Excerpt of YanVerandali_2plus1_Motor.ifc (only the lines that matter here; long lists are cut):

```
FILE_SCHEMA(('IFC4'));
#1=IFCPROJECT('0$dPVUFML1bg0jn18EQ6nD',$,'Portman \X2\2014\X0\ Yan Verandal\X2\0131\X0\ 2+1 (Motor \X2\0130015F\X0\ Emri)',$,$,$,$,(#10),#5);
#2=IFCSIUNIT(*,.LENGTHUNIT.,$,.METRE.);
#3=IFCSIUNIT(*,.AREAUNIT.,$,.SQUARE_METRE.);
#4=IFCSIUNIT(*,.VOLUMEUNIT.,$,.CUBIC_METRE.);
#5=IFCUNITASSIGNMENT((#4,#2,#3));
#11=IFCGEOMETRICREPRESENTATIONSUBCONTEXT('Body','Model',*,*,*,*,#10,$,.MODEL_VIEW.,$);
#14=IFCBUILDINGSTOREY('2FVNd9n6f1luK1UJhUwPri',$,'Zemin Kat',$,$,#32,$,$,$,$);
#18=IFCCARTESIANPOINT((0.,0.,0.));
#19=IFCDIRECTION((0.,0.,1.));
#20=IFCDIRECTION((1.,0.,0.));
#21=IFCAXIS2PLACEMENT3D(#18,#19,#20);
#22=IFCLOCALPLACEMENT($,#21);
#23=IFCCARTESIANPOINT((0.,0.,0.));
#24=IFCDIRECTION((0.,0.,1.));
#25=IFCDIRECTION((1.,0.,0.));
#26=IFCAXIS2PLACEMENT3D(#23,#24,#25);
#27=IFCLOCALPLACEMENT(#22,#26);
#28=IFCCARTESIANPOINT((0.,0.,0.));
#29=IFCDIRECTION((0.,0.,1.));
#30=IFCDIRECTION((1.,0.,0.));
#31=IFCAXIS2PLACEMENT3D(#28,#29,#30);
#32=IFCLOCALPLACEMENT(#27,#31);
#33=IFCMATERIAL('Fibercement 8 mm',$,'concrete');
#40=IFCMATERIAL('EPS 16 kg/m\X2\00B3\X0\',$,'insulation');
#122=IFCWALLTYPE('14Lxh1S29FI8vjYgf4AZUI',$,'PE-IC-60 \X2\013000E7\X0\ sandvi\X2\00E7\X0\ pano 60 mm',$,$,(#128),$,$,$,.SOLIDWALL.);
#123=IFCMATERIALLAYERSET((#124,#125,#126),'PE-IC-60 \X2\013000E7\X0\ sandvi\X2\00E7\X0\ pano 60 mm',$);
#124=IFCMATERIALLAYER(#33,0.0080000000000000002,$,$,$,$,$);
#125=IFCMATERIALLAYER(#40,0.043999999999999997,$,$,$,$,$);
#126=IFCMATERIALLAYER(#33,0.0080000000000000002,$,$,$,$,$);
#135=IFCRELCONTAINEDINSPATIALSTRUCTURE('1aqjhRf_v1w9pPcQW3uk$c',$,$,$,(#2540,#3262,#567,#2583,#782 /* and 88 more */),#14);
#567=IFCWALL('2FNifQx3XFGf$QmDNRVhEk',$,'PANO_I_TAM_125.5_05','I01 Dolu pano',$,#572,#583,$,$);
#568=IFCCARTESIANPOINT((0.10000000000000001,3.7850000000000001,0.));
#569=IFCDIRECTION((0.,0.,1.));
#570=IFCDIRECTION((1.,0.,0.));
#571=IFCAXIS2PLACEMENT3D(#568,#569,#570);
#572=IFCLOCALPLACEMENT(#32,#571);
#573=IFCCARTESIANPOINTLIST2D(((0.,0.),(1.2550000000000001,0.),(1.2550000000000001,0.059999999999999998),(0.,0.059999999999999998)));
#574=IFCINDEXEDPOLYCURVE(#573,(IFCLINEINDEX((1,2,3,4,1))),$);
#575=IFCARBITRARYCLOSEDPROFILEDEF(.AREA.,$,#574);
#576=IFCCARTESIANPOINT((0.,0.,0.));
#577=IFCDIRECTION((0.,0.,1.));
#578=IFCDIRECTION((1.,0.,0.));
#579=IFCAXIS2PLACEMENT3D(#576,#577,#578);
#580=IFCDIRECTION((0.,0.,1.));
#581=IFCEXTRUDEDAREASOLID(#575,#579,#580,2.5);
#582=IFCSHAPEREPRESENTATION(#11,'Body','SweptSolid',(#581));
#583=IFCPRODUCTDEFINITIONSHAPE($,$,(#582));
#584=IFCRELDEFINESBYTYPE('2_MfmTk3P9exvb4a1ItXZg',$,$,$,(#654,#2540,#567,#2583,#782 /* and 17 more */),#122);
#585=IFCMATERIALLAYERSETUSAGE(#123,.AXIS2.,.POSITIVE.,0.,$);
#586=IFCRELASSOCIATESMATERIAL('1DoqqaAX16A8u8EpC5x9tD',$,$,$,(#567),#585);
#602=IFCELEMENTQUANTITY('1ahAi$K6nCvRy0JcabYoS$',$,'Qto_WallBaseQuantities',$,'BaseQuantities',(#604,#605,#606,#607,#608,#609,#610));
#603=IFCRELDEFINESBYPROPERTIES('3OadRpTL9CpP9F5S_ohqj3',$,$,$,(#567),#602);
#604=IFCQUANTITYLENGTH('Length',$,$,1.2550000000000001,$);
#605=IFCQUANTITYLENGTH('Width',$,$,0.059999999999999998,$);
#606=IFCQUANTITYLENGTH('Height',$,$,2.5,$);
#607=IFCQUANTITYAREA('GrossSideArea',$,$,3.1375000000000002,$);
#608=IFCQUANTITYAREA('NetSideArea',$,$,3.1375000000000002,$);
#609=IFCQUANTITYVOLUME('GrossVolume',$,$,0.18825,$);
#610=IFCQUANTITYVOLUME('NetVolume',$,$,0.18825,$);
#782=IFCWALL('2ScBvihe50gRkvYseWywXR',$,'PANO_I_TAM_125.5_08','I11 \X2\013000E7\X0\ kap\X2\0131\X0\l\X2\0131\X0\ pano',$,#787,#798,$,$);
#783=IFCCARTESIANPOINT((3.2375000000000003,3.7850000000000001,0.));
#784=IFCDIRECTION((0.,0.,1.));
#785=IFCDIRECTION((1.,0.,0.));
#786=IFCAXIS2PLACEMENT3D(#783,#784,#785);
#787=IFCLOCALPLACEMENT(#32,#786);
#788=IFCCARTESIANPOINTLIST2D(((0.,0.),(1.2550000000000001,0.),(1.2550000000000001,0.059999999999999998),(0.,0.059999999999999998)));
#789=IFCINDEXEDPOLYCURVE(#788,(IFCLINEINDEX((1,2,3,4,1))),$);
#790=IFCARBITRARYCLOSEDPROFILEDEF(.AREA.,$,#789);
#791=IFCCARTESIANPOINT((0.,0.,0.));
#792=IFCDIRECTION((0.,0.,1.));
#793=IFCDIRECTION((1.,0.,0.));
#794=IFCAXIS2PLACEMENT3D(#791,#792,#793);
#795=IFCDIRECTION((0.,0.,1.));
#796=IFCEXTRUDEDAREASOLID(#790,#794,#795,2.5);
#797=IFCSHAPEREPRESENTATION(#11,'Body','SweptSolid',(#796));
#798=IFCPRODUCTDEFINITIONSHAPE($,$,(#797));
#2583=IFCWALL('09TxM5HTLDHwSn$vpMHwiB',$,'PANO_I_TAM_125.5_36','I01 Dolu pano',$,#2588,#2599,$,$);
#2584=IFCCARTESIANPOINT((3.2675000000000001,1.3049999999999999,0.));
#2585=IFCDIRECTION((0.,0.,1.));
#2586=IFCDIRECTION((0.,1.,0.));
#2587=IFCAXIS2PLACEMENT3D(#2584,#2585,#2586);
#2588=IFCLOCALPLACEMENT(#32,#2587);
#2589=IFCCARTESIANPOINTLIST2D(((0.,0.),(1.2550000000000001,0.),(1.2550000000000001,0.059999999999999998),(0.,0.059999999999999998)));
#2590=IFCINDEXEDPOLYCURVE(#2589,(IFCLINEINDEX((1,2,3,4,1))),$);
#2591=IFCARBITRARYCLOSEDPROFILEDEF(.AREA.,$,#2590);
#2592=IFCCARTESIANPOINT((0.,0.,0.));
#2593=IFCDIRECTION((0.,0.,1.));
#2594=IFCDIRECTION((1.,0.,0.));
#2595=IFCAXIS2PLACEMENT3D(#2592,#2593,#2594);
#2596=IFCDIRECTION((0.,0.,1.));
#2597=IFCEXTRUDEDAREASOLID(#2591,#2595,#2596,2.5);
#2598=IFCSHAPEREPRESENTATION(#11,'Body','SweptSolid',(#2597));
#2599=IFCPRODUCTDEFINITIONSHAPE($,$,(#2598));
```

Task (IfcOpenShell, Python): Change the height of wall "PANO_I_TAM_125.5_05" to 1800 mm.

```python
import ifcopenshell
import ifcopenshell.api.pset
import ifcopenshell.geom
import ifcopenshell.util.element
import ifcopenshell.util.representation
import ifcopenshell.util.shape
import ifcopenshell.util.unit

model = ifcopenshell.open("YanVerandali_2plus1_Motor.ifc")
unit_scale = ifcopenshell.util.unit.calculate_unit_scale(model)
area_scale = ifcopenshell.util.unit.calculate_unit_scale(model, "AREAUNIT")
volume_scale = ifcopenshell.util.unit.calculate_unit_scale(model, "VOLUMEUNIT")
settings = ifcopenshell.geom.settings()


def volume(element):
    """Net volume in cubic metres, openings subtracted."""
    shape = ifcopenshell.geom.create_shape(settings, element)
    return ifcopenshell.util.shape.get_volume(shape.geometry)


wall = model.by_id(567)
before = volume(wall)

body = ifcopenshell.util.representation.get_representation(wall, "Model", "Body")
solid = body.Items[0]
old_height = solid.Depth
solid.Depth = 1.8
after = volume(wall)
thickness = 0.06  # wall thickness in metres

# Update the stored height, areas and volumes.
qto = model.by_id(ifcopenshell.util.element.get_pset(wall, "Qto_WallBaseQuantities", should_inherit=False)["id"])
ifcopenshell.api.pset.edit_qto(model, qto=qto, properties={
    "Height": solid.Depth,
    "GrossSideArea": ifcopenshell.util.element.get_pset(wall, "Qto_WallBaseQuantities", "GrossSideArea") * solid.Depth / old_height,
    "NetSideArea": after / thickness / area_scale,
    "GrossVolume": ifcopenshell.util.element.get_pset(wall, "Qto_WallBaseQuantities", "GrossVolume") * solid.Depth / old_height,
    "NetVolume": after / volume_scale,
})

print(f"height {old_height:g} -> {solid.Depth:g}, volume {before:.3f} -> {after:.3f} m3")

model.write("YanVerandali_2plus1_Motor_edited.ifc")
```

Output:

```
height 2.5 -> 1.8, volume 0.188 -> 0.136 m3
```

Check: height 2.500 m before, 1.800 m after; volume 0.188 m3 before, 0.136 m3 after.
